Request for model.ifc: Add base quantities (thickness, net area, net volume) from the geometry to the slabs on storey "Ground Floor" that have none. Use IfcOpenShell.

First a look at what the model holds.

```python
import ifcopenshell
import ifcopenshell.util.element
import ifcopenshell.util.unit

model = ifcopenshell.open("model.ifc")
print(model.schema)
for unit_type in ("LENGTHUNIT", "AREAUNIT", "VOLUMEUNIT"):
    print(unit_type, ifcopenshell.util.unit.calculate_unit_scale(model, unit_type))
storey = next(s for s in model.by_type("IfcBuildingStorey") if s.Name == "Ground Floor")
slabs = [e for e in ifcopenshell.util.element.get_decomposition(storey) if e.is_a("IfcSlab")]
for e in sorted(slabs, key=lambda e: e.id()):
    print(e.id(), e.is_a(), e.Name, list(ifcopenshell.util.element.get_psets(e, qtos_only=True)), sep=" | ")
```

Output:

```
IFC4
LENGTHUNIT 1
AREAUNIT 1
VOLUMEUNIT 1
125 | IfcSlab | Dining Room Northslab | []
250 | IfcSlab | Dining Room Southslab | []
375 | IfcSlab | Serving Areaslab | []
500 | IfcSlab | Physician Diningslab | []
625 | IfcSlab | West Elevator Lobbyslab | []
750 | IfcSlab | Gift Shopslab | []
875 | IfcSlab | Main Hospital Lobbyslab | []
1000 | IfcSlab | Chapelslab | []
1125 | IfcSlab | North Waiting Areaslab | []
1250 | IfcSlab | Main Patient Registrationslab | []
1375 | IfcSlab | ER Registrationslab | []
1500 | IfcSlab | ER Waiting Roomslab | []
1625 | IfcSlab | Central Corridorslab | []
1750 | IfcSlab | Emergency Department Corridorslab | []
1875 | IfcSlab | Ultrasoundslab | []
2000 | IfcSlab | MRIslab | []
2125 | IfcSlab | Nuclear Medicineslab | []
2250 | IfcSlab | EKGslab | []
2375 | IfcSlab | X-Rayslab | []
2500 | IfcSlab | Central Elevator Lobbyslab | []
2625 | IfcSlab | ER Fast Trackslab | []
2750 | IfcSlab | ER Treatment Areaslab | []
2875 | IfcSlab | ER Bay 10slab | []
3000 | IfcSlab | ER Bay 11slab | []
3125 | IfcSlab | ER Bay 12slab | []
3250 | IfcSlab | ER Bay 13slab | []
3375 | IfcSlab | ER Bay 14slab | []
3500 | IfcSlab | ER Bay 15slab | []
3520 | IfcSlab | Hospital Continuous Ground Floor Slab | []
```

```python
import ifcopenshell
import ifcopenshell.api.pset
import ifcopenshell.geom
import ifcopenshell.util.element
import ifcopenshell.util.shape
import ifcopenshell.util.unit

model = ifcopenshell.open("model.ifc")
unit_scale = ifcopenshell.util.unit.calculate_unit_scale(model)
area_scale = ifcopenshell.util.unit.calculate_unit_scale(model, "AREAUNIT")
volume_scale = ifcopenshell.util.unit.calculate_unit_scale(model, "VOLUMEUNIT")
settings = ifcopenshell.geom.settings()

storey = next(s for s in model.by_type("IfcBuildingStorey") if s.Name == "Ground Floor")
slabs = [e for e in ifcopenshell.util.element.get_decomposition(storey) if e.is_a("IfcSlab")]

for e in sorted(slabs, key=lambda e: e.id()):
    if ifcopenshell.util.element.get_psets(e, qtos_only=True, should_inherit=False):
        continue
    # Geometry comes back in metres, in the element's own axes.
    shape = ifcopenshell.geom.create_shape(settings, e)
    values = {
        "Width": ifcopenshell.util.shape.get_z(shape.geometry) / unit_scale,
        "NetArea": ifcopenshell.util.shape.get_footprint_area(shape.geometry) / area_scale,
        "NetVolume": ifcopenshell.util.shape.get_volume(shape.geometry) / volume_scale,
    }
    qto = ifcopenshell.api.pset.add_qto(model, product=e, name="Qto_SlabBaseQuantities")
    ifcopenshell.api.pset.edit_qto(model, qto=qto, properties=values)
    print(e.id(), {k: round(v, 3) for k, v in values.items()})

model.write("model_rev.ifc")
```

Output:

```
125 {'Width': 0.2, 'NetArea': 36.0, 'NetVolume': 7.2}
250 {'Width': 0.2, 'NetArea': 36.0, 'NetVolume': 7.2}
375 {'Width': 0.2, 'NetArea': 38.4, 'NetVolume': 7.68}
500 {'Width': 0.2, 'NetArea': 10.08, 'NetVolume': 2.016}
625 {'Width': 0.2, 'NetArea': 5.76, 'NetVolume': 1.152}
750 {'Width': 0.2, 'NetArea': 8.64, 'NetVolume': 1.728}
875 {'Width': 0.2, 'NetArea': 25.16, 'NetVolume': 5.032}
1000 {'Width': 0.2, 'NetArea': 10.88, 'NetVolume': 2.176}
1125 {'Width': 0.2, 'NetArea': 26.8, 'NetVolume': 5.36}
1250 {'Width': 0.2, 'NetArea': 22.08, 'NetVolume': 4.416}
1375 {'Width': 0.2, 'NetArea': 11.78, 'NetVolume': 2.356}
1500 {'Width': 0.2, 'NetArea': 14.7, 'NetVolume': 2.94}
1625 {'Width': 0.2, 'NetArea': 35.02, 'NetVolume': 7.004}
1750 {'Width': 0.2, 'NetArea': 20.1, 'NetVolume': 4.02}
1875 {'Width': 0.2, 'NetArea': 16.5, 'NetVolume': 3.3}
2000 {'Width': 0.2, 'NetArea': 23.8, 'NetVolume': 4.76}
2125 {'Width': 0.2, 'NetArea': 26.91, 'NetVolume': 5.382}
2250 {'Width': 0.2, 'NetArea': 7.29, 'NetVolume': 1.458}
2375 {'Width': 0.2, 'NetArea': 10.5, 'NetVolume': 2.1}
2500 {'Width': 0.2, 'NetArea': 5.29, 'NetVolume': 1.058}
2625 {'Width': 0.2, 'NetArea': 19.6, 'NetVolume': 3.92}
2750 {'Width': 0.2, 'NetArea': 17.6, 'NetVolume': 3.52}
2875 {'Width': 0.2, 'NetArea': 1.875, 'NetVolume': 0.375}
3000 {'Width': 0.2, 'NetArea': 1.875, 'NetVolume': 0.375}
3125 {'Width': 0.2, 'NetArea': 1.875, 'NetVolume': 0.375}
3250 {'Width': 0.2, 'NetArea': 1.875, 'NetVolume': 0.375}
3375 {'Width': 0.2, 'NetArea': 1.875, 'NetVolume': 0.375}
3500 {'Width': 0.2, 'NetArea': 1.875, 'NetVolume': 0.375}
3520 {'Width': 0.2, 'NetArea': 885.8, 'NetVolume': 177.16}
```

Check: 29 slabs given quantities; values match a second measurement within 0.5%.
